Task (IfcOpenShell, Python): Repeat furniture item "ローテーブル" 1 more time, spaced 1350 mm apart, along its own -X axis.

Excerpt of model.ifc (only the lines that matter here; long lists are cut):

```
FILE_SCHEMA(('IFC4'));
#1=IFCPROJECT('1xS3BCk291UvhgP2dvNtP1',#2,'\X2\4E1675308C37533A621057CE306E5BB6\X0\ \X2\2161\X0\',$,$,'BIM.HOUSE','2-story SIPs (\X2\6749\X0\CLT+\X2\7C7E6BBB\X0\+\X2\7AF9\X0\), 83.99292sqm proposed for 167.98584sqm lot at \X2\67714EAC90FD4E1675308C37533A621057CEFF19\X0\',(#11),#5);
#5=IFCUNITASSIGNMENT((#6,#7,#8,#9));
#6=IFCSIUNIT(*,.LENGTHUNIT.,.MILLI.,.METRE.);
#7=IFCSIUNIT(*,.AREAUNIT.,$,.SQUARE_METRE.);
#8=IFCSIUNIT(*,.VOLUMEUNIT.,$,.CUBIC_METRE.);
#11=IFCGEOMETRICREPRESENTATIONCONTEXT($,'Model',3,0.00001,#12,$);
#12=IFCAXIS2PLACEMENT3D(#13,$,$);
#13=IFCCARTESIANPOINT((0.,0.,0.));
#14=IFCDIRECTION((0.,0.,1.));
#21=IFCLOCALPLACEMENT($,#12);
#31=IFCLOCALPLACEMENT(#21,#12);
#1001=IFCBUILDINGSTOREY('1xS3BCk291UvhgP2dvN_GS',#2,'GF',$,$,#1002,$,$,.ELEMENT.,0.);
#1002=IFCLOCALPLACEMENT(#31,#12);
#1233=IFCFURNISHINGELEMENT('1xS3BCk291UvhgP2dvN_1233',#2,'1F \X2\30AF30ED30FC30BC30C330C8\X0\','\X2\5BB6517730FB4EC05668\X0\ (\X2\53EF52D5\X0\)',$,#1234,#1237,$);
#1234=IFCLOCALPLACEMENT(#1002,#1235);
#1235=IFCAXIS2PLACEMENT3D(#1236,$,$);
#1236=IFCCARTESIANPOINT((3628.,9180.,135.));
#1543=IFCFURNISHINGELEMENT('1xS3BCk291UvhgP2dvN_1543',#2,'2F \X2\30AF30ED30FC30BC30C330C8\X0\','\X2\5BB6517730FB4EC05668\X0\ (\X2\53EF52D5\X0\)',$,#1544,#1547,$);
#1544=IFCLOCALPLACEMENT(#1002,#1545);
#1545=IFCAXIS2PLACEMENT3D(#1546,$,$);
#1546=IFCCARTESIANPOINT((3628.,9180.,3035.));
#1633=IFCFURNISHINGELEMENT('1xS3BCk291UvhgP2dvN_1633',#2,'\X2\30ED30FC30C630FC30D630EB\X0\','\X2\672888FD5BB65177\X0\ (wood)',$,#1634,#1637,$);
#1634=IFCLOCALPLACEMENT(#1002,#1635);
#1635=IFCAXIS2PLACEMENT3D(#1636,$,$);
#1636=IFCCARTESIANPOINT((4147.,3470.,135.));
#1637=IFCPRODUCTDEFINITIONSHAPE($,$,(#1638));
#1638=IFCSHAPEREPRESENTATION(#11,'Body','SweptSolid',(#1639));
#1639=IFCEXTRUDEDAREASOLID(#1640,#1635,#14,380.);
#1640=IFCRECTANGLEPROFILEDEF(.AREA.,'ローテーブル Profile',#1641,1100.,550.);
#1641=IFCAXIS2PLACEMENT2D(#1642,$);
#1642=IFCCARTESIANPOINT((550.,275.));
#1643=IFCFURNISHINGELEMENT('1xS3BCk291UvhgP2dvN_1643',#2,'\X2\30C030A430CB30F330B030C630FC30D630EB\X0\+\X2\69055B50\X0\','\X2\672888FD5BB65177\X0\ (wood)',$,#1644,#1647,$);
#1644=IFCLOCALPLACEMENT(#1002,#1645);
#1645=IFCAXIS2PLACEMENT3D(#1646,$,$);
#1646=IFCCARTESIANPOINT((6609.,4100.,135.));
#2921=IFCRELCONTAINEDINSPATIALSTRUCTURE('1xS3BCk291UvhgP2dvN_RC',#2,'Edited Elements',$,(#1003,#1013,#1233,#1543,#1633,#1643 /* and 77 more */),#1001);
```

```python
import ifcopenshell
import ifcopenshell.api.geometry
import ifcopenshell.api.root
import ifcopenshell.util.element
import ifcopenshell.util.placement
import ifcopenshell.util.unit

model = ifcopenshell.open("model.ifc")
unit_scale = ifcopenshell.util.unit.calculate_unit_scale(model)


def reuse_history(source, copy):
    """copy_class also copies each property set's owner history, people and application; keep the originals."""
    for rel in copy.IsDefinedBy:
        if rel.is_a("IfcRelDefinesByProperties") and (history := rel.RelatingPropertyDefinition.OwnerHistory):
            rel.RelatingPropertyDefinition.OwnerHistory = source.OwnerHistory
            ifcopenshell.util.element.remove_deep2(model, history)


source = model.by_id(1633)
base = ifcopenshell.util.placement.get_local_placement(source.ObjectPlacement)
step = -base[:3, 0] * 1.35 / unit_scale

for i in range(1, 2):
    copy = ifcopenshell.api.root.copy_class(model, product=source)
    copy.Representation = ifcopenshell.util.element.copy_deep(
        model, source.Representation, exclude=["IfcGeometricRepresentationContext", "IfcRepresentationMap"]
    )
    reuse_history(source, copy)
    matrix = base.copy()
    matrix[:3, 3] += i * step
    print("added at", matrix[:3, 3].round(3) + 0.0)
    ifcopenshell.api.geometry.edit_object_placement(model, product=copy, matrix=matrix, is_si=False)

model.write("model_updated.ifc")
```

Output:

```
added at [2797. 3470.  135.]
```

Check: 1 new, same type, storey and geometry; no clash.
